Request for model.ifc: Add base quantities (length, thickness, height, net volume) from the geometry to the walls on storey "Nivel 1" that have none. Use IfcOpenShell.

First a look at what the model holds.

```python
import ifcopenshell
import ifcopenshell.util.element
import ifcopenshell.util.unit

model = ifcopenshell.open("model.ifc")
print(model.schema)
for unit_type in ("LENGTHUNIT", "AREAUNIT", "VOLUMEUNIT"):
    print(unit_type, ifcopenshell.util.unit.calculate_unit_scale(model, unit_type))
storey = next(s for s in model.by_type("IfcBuildingStorey") if s.Name == "Nivel 1")
walls = [e for e in ifcopenshell.util.element.get_decomposition(storey) if e.is_a("IfcWall")]
for e in sorted(walls, key=lambda e: e.id()):
    print(e.id(), e.is_a(), e.Name, list(ifcopenshell.util.element.get_psets(e, qtos_only=True)), sep=" | ")
```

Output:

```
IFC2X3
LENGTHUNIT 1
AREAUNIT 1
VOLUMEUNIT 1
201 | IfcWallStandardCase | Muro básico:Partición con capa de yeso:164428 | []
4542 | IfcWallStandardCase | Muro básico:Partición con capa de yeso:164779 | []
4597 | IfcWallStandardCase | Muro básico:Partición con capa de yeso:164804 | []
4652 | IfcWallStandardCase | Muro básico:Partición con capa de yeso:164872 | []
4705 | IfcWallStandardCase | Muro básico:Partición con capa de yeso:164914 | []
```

```python
import ifcopenshell
import ifcopenshell.api.pset
import ifcopenshell.geom
import ifcopenshell.util.element
import ifcopenshell.util.shape
import ifcopenshell.util.unit

model = ifcopenshell.open("model.ifc")
unit_scale = ifcopenshell.util.unit.calculate_unit_scale(model)
volume_scale = ifcopenshell.util.unit.calculate_unit_scale(model, "VOLUMEUNIT")
settings = ifcopenshell.geom.settings()

storey = next(s for s in model.by_type("IfcBuildingStorey") if s.Name == "Nivel 1")
walls = [e for e in ifcopenshell.util.element.get_decomposition(storey) if e.is_a("IfcWall")]

for e in sorted(walls, key=lambda e: e.id()):
    if ifcopenshell.util.element.get_psets(e, qtos_only=True, should_inherit=False):
        continue
    # Geometry comes back in metres, in the element's own axes.
    shape = ifcopenshell.geom.create_shape(settings, e)
    values = {
        "Length": ifcopenshell.util.shape.get_x(shape.geometry) / unit_scale,
        "Width": ifcopenshell.util.shape.get_y(shape.geometry) / unit_scale,
        "Height": ifcopenshell.util.shape.get_z(shape.geometry) / unit_scale,
        "NetVolume": ifcopenshell.util.shape.get_volume(shape.geometry) / volume_scale,
    }
    qto = ifcopenshell.api.pset.add_qto(model, product=e, name="BaseQuantities")
    ifcopenshell.api.pset.edit_qto(model, qto=qto, properties=values)
    print(e.id(), {k: round(v, 3) for k, v in values.items()})

model.write("model-out.ifc")
```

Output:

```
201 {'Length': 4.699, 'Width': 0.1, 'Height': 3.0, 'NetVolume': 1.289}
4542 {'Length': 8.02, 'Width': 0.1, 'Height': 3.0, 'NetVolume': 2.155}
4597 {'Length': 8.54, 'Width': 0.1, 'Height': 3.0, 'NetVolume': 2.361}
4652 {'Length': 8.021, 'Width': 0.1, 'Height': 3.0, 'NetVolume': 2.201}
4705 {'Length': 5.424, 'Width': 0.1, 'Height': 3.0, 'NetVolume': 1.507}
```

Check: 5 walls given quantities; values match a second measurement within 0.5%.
